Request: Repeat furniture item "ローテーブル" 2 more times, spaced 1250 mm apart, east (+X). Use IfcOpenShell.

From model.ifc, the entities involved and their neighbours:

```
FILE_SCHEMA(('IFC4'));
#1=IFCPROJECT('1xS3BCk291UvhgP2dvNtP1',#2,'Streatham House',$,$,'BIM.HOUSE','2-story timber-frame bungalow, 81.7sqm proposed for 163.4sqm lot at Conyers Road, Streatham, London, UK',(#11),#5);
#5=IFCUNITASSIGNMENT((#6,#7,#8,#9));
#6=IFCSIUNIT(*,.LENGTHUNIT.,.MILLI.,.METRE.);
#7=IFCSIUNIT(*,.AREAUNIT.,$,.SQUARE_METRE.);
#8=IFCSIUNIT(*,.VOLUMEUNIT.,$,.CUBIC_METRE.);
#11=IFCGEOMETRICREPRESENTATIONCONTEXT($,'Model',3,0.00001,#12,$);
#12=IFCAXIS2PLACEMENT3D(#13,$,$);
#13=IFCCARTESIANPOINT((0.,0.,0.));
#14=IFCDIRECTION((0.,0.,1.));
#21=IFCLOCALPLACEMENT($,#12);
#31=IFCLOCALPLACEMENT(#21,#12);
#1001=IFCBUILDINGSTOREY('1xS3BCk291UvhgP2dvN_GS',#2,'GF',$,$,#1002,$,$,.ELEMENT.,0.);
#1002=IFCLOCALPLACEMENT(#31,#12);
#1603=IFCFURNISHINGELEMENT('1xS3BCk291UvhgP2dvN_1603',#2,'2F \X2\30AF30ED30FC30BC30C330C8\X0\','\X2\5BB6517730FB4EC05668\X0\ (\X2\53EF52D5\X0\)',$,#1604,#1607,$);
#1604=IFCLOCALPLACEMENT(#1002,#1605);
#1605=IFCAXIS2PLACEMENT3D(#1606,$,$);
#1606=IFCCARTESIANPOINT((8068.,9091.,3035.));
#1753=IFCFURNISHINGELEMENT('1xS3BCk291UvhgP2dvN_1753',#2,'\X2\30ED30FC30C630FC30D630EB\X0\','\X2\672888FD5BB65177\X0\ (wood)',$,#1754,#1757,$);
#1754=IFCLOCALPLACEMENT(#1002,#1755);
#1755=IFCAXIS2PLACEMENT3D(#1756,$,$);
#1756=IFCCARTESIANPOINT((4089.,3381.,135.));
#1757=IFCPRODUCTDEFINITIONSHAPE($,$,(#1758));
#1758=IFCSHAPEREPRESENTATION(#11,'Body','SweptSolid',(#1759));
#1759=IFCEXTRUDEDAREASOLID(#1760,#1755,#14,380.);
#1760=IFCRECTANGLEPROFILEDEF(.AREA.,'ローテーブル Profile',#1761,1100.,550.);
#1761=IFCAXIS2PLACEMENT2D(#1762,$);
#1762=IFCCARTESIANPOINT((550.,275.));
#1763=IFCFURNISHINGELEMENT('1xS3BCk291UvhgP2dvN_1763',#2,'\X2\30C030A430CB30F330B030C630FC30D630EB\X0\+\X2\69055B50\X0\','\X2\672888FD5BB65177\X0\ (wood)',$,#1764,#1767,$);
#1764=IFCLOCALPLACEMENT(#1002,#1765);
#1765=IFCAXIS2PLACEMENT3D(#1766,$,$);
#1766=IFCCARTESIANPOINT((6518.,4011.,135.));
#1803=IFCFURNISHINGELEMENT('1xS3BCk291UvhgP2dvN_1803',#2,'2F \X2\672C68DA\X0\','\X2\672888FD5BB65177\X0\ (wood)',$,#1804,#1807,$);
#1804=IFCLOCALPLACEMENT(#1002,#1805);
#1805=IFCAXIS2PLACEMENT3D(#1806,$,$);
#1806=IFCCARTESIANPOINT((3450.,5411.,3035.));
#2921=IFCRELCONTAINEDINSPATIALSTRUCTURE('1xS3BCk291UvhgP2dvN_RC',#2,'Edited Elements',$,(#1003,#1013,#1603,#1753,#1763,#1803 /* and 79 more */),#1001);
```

```python
import numpy as np
import ifcopenshell
import ifcopenshell.api.geometry
import ifcopenshell.api.root
import ifcopenshell.util.element
import ifcopenshell.util.placement
import ifcopenshell.util.unit

model = ifcopenshell.open("model.ifc")
unit_scale = ifcopenshell.util.unit.calculate_unit_scale(model)


def reuse_history(source, copy):
    """copy_class also copies each property set's owner history, people and application; keep the originals."""
    for rel in copy.IsDefinedBy:
        if rel.is_a("IfcRelDefinesByProperties") and (history := rel.RelatingPropertyDefinition.OwnerHistory):
            rel.RelatingPropertyDefinition.OwnerHistory = source.OwnerHistory
            ifcopenshell.util.element.remove_deep2(model, history)


source = model.by_id(1753)
base = ifcopenshell.util.placement.get_local_placement(source.ObjectPlacement)
step = np.array([1.0, 0.0, 0.0]) * 1.25 / unit_scale

for i in range(1, 3):
    copy = ifcopenshell.api.root.copy_class(model, product=source)
    copy.Representation = ifcopenshell.util.element.copy_deep(
        model, source.Representation, exclude=["IfcGeometricRepresentationContext", "IfcRepresentationMap"]
    )
    reuse_history(source, copy)
    matrix = base.copy()
    matrix[:3, 3] += i * step
    print("added at", matrix[:3, 3].round(3) + 0.0)
    ifcopenshell.api.geometry.edit_object_placement(model, product=copy, matrix=matrix, is_si=False)

model.write("model_v2.ifc")
```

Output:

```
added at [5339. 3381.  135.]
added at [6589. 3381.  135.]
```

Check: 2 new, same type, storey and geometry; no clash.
